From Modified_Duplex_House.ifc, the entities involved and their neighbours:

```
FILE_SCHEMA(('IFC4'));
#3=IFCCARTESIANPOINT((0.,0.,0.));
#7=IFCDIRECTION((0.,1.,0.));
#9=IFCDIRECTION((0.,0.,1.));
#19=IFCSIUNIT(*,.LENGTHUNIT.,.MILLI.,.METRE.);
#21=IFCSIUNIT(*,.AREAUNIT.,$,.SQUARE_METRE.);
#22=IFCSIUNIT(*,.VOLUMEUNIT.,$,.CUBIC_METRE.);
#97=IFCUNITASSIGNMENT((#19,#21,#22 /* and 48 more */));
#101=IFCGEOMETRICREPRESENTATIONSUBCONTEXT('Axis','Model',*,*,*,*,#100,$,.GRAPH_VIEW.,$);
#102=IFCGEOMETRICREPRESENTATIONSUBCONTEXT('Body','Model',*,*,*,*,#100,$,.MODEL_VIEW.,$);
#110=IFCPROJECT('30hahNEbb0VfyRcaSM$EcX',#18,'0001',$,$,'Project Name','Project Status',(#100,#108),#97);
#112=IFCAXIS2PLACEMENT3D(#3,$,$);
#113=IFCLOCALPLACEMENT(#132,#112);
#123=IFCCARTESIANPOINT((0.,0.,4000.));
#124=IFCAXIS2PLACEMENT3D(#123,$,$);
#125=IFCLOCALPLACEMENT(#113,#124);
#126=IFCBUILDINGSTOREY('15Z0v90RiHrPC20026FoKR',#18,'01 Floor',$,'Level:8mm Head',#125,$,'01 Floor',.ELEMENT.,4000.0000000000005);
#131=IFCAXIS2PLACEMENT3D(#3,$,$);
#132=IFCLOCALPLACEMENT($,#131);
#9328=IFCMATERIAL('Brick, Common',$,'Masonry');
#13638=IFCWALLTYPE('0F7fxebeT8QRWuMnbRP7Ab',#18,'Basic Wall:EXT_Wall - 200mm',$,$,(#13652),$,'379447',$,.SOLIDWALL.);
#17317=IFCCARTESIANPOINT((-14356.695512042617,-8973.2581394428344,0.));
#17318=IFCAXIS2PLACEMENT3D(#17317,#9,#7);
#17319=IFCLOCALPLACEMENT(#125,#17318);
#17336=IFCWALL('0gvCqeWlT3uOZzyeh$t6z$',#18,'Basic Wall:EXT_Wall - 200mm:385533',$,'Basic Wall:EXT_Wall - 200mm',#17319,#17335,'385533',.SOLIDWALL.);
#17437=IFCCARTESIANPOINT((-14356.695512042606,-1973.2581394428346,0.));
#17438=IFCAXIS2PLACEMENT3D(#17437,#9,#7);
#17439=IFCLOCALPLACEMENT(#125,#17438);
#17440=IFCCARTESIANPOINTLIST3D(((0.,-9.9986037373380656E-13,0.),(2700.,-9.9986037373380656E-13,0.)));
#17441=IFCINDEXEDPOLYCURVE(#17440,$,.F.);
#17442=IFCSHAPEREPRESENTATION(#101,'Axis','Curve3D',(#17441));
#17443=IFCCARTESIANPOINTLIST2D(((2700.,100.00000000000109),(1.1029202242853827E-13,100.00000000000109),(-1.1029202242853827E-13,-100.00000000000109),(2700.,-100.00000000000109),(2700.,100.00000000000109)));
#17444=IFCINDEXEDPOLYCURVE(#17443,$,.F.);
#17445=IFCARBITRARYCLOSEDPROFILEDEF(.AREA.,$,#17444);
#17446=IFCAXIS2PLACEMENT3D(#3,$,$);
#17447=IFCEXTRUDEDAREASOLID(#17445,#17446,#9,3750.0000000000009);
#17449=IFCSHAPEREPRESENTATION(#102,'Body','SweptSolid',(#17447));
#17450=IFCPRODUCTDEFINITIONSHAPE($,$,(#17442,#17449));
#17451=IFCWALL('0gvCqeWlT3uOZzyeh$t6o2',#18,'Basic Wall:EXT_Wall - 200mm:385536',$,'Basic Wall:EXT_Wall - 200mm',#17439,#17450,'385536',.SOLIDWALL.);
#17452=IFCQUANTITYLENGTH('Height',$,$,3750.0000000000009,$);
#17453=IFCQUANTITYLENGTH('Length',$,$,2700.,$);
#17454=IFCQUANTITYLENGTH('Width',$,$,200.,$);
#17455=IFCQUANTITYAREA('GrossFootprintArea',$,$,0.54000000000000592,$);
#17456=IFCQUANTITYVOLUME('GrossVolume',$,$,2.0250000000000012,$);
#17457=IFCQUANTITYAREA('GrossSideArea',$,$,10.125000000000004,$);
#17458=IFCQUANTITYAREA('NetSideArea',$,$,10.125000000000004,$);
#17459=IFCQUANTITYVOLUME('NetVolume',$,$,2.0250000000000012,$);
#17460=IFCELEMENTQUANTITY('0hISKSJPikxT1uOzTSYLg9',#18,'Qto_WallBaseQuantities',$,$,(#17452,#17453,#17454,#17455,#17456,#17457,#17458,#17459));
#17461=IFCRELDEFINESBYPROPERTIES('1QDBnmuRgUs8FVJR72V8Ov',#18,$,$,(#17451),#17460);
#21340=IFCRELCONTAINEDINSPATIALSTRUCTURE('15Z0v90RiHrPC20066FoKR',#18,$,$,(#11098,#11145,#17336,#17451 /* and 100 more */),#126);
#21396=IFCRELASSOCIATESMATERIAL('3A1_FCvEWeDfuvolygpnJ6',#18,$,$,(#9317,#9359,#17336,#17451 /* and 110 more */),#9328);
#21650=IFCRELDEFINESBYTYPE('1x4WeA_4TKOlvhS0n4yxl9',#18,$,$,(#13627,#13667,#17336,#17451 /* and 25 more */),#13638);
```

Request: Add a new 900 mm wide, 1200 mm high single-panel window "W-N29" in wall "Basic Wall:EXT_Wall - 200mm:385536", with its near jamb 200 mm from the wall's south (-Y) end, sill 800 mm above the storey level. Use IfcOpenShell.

```python
import numpy as np
import ifcopenshell
import ifcopenshell.api.feature
import ifcopenshell.api.geometry
import ifcopenshell.api.pset
import ifcopenshell.api.root
import ifcopenshell.api.spatial
import ifcopenshell.geom
import ifcopenshell.util.element
import ifcopenshell.util.placement
import ifcopenshell.util.representation
import ifcopenshell.util.shape
import ifcopenshell.util.unit

model = ifcopenshell.open("Modified_Duplex_House.ifc")
unit_scale = ifcopenshell.util.unit.calculate_unit_scale(model)
area_scale = ifcopenshell.util.unit.calculate_unit_scale(model, "AREAUNIT")
volume_scale = ifcopenshell.util.unit.calculate_unit_scale(model, "VOLUMEUNIT")
settings = ifcopenshell.geom.settings()


def volume(element):
    """Net volume in cubic metres, openings subtracted."""
    shape = ifcopenshell.geom.create_shape(settings, element)
    return ifcopenshell.util.shape.get_volume(shape.geometry)


wall = model.by_guid("0gvCqeWlT3uOZzyeh$t6o2")
storey = ifcopenshell.util.element.get_container(wall, ifc_class="IfcBuildingStorey")
context = ifcopenshell.util.representation.get_context(model, "Model", "Body", "MODEL_VIEW")
before = volume(wall)

width, height, from_end, sill = 0.9, 1.2, 0.2, 0.8  # metres

# The wall runs along its own X axis, and the end named is its -X end.
wall_shape = ifcopenshell.geom.create_shape(settings, wall)
x, y, z = ifcopenshell.util.shape.get_vertices(wall_shape.geometry).T
start = x.min() + from_end
face, thickness = float(y.min()), float(y.max() - y.min())
wall_matrix = ifcopenshell.util.placement.get_local_placement(wall.ObjectPlacement)
level = ifcopenshell.util.placement.get_local_placement(storey.ObjectPlacement)[2, 3]


def in_wall(x, y):
    """Placement at x, y metres in the wall's axes, at sill height."""
    matrix = wall_matrix.copy()
    matrix[:, 3] = wall_matrix @ np.array([x / unit_scale, y / unit_scale, 0.0, 1.0])
    matrix[2, 3] = level + sill / unit_scale
    return matrix


# Opening: a box that overshoots both wall faces by 50 mm.
opening = ifcopenshell.api.root.create_entity(model, ifc_class="IfcOpeningElement", predefined_type="OPENING")
box = ifcopenshell.api.geometry.add_wall_representation(
    model, context=context, length=width, height=height, thickness=thickness + 0.1
)
ifcopenshell.api.geometry.assign_representation(model, product=opening, representation=box)
ifcopenshell.api.geometry.edit_object_placement(model, product=opening, matrix=in_wall(start, face - 0.05), is_si=False)
ifcopenshell.api.feature.add_feature(model, feature=opening, element=wall)

window = ifcopenshell.api.root.create_entity(model, ifc_class="IfcWindow", name="W-N29", predefined_type="WINDOW")
window.OverallWidth, window.OverallHeight = width / unit_scale, height / unit_scale
window.PartitioningType = "SINGLE_PANEL"
body = ifcopenshell.api.geometry.add_window_representation(
    model,
    context=context,
    overall_width=window.OverallWidth,
    overall_height=window.OverallHeight,
    partition_type="SINGLE_PANEL",
)
ifcopenshell.api.geometry.assign_representation(model, product=window, representation=body)
ifcopenshell.api.spatial.assign_container(model, products=[window], relating_structure=storey)
ifcopenshell.api.feature.add_filling(model, opening=opening, element=window)

# Centre the window in the wall's thickness.
ifcopenshell.api.geometry.edit_object_placement(model, product=window, matrix=in_wall(start, face), is_si=False)
window_shape = ifcopenshell.geom.create_shape(settings, window)
depth = ifcopenshell.util.shape.get_vertices(window_shape.geometry)[:, 1]
offset = face + thickness / 2 - (depth.min() + depth.max()) / 2
ifcopenshell.api.geometry.edit_object_placement(model, product=window, matrix=in_wall(start, offset), is_si=False)

after = volume(wall)

# Update the wall's stored quantities.
qto = model.by_id(ifcopenshell.util.element.get_pset(wall, "Qto_WallBaseQuantities", should_inherit=False)["id"])
ifcopenshell.api.pset.edit_qto(model, qto=qto, properties={
    "NetSideArea": after / thickness / area_scale,
    "NetVolume": after / volume_scale,
})

print(f"wall volume {before:.3f} -> {after:.3f} m3")

model.write("Modified_Duplex_House_v2.ifc")
```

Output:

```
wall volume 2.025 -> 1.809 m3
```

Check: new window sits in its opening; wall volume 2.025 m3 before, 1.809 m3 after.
